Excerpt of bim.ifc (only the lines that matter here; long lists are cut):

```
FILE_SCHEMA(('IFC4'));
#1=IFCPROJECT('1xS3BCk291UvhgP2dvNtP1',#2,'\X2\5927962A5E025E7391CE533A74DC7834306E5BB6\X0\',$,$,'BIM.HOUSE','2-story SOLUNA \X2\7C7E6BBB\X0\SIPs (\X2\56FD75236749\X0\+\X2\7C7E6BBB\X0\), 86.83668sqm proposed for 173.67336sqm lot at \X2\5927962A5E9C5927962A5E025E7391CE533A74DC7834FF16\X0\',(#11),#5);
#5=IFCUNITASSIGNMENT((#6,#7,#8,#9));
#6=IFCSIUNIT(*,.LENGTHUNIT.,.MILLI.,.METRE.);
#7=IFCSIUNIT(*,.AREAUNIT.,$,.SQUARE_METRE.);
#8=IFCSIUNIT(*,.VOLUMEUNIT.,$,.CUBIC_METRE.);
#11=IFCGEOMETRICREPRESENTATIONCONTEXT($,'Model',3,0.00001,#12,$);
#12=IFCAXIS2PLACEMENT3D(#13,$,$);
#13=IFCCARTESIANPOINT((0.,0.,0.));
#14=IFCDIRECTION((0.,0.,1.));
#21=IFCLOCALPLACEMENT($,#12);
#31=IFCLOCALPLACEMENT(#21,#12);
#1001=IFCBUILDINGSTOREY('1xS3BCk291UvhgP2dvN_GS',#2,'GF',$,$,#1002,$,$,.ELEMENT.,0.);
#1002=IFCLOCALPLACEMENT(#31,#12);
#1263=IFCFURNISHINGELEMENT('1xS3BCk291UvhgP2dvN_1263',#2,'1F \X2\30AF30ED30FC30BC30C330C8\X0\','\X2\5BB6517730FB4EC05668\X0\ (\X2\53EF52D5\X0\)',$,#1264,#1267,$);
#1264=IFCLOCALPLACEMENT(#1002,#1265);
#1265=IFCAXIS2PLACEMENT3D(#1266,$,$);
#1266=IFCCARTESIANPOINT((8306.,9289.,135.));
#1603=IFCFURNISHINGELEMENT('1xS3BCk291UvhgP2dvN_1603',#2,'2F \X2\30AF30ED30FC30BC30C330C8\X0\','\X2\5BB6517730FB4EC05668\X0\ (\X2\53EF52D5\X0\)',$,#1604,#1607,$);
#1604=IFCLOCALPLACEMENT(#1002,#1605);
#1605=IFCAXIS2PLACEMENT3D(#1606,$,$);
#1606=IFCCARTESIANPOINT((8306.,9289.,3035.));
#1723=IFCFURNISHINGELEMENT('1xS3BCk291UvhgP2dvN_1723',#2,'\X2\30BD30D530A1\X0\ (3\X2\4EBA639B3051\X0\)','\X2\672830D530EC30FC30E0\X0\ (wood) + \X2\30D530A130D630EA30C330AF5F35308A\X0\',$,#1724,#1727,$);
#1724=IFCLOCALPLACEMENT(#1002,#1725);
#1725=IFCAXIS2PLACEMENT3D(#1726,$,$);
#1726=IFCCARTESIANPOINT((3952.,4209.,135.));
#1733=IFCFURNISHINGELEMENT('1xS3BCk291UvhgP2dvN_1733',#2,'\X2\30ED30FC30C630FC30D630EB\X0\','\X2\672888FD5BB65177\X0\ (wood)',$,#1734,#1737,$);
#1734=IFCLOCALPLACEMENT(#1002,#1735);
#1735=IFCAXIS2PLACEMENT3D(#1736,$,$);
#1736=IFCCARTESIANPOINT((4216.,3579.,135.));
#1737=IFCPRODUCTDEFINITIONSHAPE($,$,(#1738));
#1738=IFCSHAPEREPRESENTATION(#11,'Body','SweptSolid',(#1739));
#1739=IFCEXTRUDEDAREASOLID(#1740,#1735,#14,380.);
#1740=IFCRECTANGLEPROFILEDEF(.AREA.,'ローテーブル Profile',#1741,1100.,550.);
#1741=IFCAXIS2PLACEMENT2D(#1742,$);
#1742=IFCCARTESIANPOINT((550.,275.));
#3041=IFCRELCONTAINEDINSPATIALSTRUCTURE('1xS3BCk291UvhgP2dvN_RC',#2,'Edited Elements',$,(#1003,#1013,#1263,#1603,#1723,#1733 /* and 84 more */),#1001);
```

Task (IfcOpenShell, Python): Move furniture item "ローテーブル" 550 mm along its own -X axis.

```python
import ifcopenshell
import ifcopenshell.api.geometry
import ifcopenshell.util.placement

model = ifcopenshell.open("bim.ifc")

item = model.by_guid("1xS3BCk291UvhgP2dvN_1733")
matrix = ifcopenshell.util.placement.get_local_placement(item.ObjectPlacement)
matrix[:3, 3] -= matrix[:3, 0] * 550.0
ifcopenshell.api.geometry.edit_object_placement(model, product=item, matrix=matrix, is_si=False)

print(ifcopenshell.util.placement.get_local_placement(item.ObjectPlacement).round(3) + 0.0)

model.write("bim-out.ifc")
```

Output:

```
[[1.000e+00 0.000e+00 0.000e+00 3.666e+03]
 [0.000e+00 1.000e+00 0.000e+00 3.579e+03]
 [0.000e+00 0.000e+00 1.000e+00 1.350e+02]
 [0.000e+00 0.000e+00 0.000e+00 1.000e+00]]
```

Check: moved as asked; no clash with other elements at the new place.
